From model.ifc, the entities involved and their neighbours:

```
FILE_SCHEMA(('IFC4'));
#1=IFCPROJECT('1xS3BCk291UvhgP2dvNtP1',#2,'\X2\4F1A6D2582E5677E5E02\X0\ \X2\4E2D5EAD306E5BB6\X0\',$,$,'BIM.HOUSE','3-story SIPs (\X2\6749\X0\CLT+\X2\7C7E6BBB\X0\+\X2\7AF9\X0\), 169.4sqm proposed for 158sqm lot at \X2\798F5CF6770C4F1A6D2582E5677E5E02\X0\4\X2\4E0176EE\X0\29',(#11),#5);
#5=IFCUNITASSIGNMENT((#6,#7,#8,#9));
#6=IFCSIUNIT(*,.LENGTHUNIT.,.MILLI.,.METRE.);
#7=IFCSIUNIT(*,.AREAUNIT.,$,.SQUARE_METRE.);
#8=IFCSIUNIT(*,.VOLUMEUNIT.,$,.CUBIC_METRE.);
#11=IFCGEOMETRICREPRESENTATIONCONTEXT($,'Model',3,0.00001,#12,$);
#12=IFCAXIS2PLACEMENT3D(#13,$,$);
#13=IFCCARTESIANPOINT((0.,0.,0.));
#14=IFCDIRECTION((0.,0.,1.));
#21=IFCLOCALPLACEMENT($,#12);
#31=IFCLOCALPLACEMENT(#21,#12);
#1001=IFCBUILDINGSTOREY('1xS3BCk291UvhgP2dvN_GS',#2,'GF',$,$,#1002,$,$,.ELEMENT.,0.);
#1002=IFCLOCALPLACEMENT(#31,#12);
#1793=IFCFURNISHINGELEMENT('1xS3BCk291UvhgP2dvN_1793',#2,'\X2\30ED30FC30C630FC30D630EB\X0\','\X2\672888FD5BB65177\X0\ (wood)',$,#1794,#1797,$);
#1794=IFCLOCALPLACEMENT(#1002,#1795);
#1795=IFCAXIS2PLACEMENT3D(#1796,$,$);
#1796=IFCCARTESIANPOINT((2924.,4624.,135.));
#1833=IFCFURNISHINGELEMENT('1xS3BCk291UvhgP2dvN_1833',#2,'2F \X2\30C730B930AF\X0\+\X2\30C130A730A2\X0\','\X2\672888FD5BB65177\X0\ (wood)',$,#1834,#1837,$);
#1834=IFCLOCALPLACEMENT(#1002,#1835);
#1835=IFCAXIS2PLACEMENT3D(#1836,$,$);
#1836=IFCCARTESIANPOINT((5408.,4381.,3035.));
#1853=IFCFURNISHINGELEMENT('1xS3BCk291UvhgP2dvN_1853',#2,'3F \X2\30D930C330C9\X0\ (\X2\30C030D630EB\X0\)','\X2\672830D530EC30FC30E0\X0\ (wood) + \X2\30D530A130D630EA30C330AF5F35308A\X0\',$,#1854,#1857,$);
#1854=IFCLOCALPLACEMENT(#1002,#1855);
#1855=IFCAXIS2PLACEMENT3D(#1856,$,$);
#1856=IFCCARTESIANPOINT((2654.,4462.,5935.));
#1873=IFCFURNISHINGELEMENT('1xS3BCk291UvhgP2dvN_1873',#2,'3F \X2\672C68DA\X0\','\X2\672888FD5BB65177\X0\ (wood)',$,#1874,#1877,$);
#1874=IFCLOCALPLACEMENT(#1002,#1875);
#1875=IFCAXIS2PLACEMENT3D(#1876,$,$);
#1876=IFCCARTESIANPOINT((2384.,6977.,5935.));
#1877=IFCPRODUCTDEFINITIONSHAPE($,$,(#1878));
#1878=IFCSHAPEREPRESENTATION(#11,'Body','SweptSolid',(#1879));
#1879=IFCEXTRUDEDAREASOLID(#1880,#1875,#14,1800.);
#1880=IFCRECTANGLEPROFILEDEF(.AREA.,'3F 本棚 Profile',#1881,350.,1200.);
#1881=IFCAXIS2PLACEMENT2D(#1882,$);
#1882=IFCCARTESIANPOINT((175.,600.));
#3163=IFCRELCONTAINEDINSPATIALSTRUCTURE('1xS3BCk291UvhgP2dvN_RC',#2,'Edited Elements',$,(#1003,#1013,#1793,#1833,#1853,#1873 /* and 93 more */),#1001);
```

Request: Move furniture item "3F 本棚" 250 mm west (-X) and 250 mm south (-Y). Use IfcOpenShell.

```python
import ifcopenshell
import ifcopenshell.api.geometry
import ifcopenshell.util.placement

model = ifcopenshell.open("model.ifc")

item = model.by_id(1873)
matrix = ifcopenshell.util.placement.get_local_placement(item.ObjectPlacement)
matrix[0, 3] -= 250.0
matrix[1, 3] -= 250.0
ifcopenshell.api.geometry.edit_object_placement(model, product=item, matrix=matrix, is_si=False)

print(ifcopenshell.util.placement.get_local_placement(item.ObjectPlacement).round(3) + 0.0)

model.write("model_v2.ifc")
```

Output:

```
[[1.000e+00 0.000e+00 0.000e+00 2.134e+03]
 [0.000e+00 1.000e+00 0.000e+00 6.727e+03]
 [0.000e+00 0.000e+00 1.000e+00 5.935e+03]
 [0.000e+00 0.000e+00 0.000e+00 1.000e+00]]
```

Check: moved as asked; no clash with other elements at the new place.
